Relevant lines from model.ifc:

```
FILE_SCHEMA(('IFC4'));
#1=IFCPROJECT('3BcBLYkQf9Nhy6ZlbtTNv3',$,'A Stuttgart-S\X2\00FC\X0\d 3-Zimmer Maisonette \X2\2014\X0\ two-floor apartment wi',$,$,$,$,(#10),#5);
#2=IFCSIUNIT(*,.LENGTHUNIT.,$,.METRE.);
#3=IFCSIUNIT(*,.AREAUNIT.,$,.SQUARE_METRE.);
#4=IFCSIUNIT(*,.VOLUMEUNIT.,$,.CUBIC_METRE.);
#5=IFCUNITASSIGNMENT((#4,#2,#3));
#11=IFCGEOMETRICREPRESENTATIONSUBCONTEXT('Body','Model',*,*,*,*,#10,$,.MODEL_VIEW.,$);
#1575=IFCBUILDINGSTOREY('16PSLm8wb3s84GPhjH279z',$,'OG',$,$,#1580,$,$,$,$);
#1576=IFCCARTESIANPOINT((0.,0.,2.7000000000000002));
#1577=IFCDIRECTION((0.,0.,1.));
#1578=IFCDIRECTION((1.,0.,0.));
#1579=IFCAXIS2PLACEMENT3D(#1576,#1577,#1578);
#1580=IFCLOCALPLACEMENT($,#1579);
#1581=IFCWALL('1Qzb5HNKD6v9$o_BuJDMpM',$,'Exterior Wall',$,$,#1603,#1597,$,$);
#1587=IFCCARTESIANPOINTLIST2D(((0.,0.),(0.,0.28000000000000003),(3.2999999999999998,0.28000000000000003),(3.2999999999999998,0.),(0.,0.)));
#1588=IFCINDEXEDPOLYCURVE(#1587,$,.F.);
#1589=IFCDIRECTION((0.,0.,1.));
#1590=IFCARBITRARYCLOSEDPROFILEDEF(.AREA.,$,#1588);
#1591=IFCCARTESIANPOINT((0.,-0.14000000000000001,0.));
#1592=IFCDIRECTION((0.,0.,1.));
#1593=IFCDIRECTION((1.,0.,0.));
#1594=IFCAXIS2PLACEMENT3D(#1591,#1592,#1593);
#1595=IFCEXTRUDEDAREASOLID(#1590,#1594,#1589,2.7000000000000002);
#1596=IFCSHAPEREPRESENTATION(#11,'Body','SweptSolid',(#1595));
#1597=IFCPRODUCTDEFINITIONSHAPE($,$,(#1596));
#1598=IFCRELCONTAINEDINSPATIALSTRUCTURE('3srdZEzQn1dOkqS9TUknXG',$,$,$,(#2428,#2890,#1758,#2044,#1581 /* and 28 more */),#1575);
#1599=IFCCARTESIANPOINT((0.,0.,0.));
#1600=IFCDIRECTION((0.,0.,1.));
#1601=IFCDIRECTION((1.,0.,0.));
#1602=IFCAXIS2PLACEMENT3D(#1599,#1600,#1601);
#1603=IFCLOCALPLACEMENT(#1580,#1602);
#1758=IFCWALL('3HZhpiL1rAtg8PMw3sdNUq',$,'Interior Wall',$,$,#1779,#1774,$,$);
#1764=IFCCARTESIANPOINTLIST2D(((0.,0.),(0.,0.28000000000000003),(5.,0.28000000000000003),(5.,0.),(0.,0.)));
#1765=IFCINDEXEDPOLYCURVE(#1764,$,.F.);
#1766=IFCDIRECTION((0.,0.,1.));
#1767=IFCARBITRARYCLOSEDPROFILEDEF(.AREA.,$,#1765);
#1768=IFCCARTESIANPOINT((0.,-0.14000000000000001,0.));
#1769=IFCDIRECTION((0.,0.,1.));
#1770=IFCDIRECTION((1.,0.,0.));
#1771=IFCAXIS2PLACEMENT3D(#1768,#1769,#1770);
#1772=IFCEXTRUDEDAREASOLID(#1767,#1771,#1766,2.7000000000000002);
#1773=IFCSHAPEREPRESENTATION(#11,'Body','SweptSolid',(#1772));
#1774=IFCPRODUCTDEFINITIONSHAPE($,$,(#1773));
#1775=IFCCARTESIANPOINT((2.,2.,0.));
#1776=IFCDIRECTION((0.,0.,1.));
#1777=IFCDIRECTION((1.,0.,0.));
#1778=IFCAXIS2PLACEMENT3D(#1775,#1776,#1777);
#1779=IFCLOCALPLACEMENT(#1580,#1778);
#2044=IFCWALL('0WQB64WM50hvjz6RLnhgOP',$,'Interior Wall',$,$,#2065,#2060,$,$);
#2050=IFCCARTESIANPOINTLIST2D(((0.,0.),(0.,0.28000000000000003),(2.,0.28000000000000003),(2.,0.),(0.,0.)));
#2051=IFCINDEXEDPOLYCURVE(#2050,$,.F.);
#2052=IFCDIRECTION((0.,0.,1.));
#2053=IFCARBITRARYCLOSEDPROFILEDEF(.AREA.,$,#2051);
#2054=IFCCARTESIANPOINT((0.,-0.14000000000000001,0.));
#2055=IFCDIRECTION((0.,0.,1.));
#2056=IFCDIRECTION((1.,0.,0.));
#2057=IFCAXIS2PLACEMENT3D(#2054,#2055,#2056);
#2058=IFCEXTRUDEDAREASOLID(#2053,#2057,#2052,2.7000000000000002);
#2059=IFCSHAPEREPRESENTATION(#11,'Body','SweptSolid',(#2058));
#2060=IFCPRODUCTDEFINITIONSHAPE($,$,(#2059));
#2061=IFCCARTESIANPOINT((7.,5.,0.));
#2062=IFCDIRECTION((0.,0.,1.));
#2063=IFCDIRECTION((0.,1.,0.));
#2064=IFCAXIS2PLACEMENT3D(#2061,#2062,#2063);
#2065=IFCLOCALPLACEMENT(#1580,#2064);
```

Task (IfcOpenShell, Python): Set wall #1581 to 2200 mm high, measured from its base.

```python
import ifcopenshell
import ifcopenshell.geom
import ifcopenshell.util.representation
import ifcopenshell.util.shape

model = ifcopenshell.open("model.ifc")
settings = ifcopenshell.geom.settings()


def volume(element):
    """Net volume in cubic metres, openings subtracted."""
    shape = ifcopenshell.geom.create_shape(settings, element)
    return ifcopenshell.util.shape.get_volume(shape.geometry)


wall = model.by_id(1581)
before = volume(wall)

body = ifcopenshell.util.representation.get_representation(wall, "Model", "Body")
solid = body.Items[0]
old_height = solid.Depth
solid.Depth = 2.2
after = volume(wall)

print(f"height {old_height:g} -> {solid.Depth:g}, volume {before:.3f} -> {after:.3f} m3")

model.write("model-out.ifc")
```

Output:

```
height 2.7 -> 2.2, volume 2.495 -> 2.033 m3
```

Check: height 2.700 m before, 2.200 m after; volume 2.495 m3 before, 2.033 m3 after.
